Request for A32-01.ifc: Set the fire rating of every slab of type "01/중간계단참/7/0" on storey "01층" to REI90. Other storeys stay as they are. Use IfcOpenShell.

First a look at what the model holds.

```python
import ifcopenshell
import ifcopenshell.util.element

model = ifcopenshell.open("A32-01.ifc")
print(model.schema)
storey = next(s for s in model.by_type("IfcBuildingStorey") if s.Name == "01층")
slabs = [e for e in ifcopenshell.util.element.get_decomposition(storey) if e.is_a("IfcSlab")]
seen = {}
for e in slabs:
    element_type = ifcopenshell.util.element.get_type(e)
    key = (element_type.Name if element_type != e and element_type else None, ifcopenshell.util.element.get_pset(e, "Pset_SlabCommon", "FireRating"))
    seen[key] = seen.get(key, 0) + 1
for (name, value), count in sorted(seen.items(), key=str):
    print(count, "x", name, "|", value)
```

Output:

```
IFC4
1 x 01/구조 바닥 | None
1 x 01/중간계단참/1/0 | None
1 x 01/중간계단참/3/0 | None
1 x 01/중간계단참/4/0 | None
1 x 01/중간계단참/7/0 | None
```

```python
import ifcopenshell
import ifcopenshell.api.pset
import ifcopenshell.util.element

model = ifcopenshell.open("A32-01.ifc")

storey = next(s for s in model.by_type("IfcBuildingStorey") if s.Name == "01층")
slabs = [e for e in ifcopenshell.util.element.get_decomposition(storey) if e.is_a("IfcSlab")]

count = 0
for e in slabs:
    element_type = ifcopenshell.util.element.get_type(e)
    if element_type in (None, e) or element_type.Name != "01/중간계단참/7/0":
        continue
    # add_pset returns the element's existing set when there is one.
    pset = ifcopenshell.api.pset.add_pset(model, product=e, name="Pset_SlabCommon")
    ifcopenshell.api.pset.edit_pset(model, pset=pset, properties={"FireRating": "REI90"})
    count += 1

print(count, "slabs updated")

model.write("A32-01-out.ifc")
```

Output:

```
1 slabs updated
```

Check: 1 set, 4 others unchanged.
